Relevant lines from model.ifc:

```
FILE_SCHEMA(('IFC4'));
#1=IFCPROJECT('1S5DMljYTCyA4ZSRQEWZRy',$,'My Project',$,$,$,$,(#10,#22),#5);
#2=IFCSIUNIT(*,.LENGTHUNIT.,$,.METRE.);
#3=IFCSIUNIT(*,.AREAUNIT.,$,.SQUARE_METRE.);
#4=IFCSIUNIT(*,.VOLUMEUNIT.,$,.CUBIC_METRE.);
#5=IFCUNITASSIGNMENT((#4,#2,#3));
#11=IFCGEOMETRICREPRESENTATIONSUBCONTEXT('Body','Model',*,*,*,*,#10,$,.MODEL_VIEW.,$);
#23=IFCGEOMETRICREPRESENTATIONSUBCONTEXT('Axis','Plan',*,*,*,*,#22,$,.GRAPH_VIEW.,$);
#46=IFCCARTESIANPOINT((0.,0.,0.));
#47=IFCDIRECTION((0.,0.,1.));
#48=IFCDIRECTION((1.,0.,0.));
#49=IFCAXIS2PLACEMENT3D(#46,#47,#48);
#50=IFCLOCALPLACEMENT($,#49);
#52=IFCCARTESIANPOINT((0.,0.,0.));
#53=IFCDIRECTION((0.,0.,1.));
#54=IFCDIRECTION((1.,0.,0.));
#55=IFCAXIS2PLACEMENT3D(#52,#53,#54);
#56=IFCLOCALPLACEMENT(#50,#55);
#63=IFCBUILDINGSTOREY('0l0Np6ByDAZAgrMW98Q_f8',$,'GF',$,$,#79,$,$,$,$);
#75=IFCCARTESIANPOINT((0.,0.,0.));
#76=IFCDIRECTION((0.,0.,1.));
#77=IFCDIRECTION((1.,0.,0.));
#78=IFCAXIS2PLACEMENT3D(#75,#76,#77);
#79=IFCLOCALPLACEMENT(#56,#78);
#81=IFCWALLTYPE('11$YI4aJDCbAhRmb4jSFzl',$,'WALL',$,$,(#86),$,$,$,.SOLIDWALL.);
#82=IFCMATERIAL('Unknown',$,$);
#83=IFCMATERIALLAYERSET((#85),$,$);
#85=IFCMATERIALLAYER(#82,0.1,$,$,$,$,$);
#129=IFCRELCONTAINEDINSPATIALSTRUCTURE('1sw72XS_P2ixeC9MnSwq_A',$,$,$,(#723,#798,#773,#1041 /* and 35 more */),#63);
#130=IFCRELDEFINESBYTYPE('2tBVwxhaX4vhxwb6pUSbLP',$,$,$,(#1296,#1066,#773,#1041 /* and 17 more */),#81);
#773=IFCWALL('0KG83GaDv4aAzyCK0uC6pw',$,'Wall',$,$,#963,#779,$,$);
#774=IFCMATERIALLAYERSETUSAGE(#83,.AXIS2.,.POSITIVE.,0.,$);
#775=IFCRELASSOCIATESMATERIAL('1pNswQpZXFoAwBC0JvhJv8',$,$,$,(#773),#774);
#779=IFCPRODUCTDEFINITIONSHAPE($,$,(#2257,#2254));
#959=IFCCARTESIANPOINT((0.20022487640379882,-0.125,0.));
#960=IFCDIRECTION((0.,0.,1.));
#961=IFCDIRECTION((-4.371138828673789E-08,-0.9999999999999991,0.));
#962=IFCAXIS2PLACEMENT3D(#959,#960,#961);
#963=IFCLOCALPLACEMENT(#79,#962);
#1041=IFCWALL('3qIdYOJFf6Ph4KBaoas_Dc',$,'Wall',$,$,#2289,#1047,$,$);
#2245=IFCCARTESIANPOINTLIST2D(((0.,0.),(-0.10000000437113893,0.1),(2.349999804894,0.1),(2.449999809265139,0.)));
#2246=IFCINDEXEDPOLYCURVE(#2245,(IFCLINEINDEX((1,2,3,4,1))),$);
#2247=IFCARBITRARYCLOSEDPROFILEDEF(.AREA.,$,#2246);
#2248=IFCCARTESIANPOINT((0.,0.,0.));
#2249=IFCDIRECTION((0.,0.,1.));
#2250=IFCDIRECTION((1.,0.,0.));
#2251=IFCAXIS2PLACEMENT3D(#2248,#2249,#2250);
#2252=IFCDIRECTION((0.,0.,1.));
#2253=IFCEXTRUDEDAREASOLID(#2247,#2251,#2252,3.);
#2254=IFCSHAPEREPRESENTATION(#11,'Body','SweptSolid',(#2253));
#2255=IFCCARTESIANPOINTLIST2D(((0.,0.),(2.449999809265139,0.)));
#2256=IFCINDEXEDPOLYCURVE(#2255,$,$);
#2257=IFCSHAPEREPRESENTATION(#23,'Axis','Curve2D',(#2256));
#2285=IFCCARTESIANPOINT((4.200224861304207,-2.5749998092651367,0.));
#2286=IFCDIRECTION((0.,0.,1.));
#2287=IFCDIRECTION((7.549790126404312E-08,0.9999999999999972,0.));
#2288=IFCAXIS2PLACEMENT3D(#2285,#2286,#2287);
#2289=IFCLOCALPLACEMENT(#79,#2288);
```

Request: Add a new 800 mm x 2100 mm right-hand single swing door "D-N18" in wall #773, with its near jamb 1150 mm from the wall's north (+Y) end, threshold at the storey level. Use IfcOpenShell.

```python
import numpy as np
import ifcopenshell
import ifcopenshell.api.feature
import ifcopenshell.api.geometry
import ifcopenshell.api.root
import ifcopenshell.api.spatial
import ifcopenshell.geom
import ifcopenshell.util.element
import ifcopenshell.util.placement
import ifcopenshell.util.representation
import ifcopenshell.util.shape
import ifcopenshell.util.unit

model = ifcopenshell.open("model.ifc")
unit_scale = ifcopenshell.util.unit.calculate_unit_scale(model)
settings = ifcopenshell.geom.settings()


def volume(element):
    """Net volume in cubic metres, openings subtracted."""
    shape = ifcopenshell.geom.create_shape(settings, element)
    return ifcopenshell.util.shape.get_volume(shape.geometry)


wall = model.by_guid("0KG83GaDv4aAzyCK0uC6pw")
storey = ifcopenshell.util.element.get_container(wall, ifc_class="IfcBuildingStorey")
context = ifcopenshell.util.representation.get_context(model, "Model", "Body", "MODEL_VIEW")
before = volume(wall)

width, height, from_end, sill = 0.8, 2.1, 1.15, 0.0  # metres

# The wall runs along its own X axis, and the end named is its -X end.
wall_shape = ifcopenshell.geom.create_shape(settings, wall)
x, y, z = ifcopenshell.util.shape.get_vertices(wall_shape.geometry).T
start = x.min() + from_end
face, thickness = float(y.min()), float(y.max() - y.min())
wall_matrix = ifcopenshell.util.placement.get_local_placement(wall.ObjectPlacement)
level = ifcopenshell.util.placement.get_local_placement(storey.ObjectPlacement)[2, 3]


def in_wall(x, y):
    """Placement at x, y metres in the wall's axes, at sill height."""
    matrix = wall_matrix.copy()
    matrix[:, 3] = wall_matrix @ np.array([x / unit_scale, y / unit_scale, 0.0, 1.0])
    matrix[2, 3] = level + sill / unit_scale
    return matrix


# Opening: a box that overshoots both wall faces by 50 mm.
opening = ifcopenshell.api.root.create_entity(model, ifc_class="IfcOpeningElement", predefined_type="OPENING")
box = ifcopenshell.api.geometry.add_wall_representation(
    model, context=context, length=width, height=height, thickness=thickness + 0.1
)
ifcopenshell.api.geometry.assign_representation(model, product=opening, representation=box)
ifcopenshell.api.geometry.edit_object_placement(model, product=opening, matrix=in_wall(start, face - 0.05), is_si=False)
ifcopenshell.api.feature.add_feature(model, feature=opening, element=wall)

door = ifcopenshell.api.root.create_entity(model, ifc_class="IfcDoor", name="D-N18", predefined_type="DOOR")
door.OverallWidth, door.OverallHeight = width / unit_scale, height / unit_scale
door.OperationType = "SINGLE_SWING_RIGHT"
body = ifcopenshell.api.geometry.add_door_representation(
    model,
    context=context,
    overall_width=door.OverallWidth,
    overall_height=door.OverallHeight,
    operation_type="SINGLE_SWING_RIGHT",
    lining_properties={"LiningDepth": thickness / unit_scale, "ThresholdDepth": thickness / unit_scale},
)
ifcopenshell.api.geometry.assign_representation(model, product=door, representation=body)
ifcopenshell.api.spatial.assign_container(model, products=[door], relating_structure=storey)
ifcopenshell.api.feature.add_filling(model, opening=opening, element=door)

# The lining spans the wall, so the door starts at the wall face.
ifcopenshell.api.geometry.edit_object_placement(model, product=door, matrix=in_wall(start, face), is_si=False)

after = volume(wall)

print(f"wall volume {before:.3f} -> {after:.3f} m3")

model.write("model_updated.ifc")
```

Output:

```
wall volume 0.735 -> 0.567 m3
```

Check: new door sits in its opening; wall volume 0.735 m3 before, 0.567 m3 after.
